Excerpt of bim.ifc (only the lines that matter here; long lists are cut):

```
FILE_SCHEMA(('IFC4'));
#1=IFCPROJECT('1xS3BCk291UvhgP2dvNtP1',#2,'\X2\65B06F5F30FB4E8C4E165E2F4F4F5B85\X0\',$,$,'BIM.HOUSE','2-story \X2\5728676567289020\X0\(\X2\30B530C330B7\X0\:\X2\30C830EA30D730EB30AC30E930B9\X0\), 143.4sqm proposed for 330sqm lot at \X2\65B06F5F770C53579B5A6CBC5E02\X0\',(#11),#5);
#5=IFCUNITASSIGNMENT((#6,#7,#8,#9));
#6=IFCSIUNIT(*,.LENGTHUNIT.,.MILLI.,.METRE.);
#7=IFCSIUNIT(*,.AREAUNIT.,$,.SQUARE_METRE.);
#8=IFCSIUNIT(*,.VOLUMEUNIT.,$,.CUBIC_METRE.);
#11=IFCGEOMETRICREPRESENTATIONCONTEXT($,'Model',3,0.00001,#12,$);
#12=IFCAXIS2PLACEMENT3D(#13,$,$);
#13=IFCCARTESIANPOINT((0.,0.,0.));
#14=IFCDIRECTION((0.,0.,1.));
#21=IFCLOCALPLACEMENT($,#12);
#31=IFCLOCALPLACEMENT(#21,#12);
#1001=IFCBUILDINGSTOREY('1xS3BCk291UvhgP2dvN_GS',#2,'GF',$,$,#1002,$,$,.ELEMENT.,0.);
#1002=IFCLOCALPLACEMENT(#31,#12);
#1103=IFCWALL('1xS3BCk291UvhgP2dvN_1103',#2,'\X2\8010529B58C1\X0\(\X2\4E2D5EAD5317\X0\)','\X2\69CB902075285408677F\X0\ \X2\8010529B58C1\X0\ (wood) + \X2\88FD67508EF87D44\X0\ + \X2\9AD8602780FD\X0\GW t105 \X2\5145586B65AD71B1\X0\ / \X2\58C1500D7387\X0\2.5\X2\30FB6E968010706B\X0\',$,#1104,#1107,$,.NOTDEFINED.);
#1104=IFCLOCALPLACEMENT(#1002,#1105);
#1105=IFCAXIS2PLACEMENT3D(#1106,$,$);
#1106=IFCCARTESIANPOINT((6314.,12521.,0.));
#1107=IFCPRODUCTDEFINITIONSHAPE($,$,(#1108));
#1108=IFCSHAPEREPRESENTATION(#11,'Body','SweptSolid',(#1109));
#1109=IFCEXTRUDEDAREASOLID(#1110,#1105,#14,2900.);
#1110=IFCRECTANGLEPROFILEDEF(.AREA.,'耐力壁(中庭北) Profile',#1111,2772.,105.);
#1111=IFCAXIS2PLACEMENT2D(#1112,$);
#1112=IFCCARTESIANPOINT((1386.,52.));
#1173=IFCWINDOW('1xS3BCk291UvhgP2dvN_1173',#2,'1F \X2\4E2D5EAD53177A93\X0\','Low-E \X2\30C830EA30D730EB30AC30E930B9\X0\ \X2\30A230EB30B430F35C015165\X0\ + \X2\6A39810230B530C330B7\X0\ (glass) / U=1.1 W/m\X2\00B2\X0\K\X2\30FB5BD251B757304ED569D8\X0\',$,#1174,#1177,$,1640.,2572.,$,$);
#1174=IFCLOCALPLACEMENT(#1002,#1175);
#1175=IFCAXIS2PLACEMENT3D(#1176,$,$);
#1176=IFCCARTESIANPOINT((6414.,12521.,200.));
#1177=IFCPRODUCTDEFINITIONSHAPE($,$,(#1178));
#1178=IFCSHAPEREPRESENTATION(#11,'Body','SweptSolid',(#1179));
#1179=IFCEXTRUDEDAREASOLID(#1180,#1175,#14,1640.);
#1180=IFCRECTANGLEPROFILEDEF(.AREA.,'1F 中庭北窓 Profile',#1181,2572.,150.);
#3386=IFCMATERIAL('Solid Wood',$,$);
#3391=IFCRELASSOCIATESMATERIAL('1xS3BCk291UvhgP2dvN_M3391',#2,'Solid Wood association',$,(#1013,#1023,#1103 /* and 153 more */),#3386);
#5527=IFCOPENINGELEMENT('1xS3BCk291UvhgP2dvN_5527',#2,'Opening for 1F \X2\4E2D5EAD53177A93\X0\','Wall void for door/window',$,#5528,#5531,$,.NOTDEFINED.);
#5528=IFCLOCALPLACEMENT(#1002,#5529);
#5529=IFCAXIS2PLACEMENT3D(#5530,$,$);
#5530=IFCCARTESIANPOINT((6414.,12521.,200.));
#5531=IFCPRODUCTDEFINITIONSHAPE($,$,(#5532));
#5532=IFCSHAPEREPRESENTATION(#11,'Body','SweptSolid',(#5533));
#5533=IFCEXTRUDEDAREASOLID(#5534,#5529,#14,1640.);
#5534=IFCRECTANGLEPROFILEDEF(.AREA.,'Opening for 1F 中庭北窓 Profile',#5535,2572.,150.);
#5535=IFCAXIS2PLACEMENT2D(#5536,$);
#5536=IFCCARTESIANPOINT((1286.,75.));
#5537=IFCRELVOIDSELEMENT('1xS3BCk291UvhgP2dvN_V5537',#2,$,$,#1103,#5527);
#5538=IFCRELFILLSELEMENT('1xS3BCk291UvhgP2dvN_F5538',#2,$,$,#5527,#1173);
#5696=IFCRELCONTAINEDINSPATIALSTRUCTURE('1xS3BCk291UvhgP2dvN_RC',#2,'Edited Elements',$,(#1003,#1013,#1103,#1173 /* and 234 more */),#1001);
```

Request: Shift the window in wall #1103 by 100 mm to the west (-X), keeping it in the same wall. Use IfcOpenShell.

```python
import ifcopenshell
import ifcopenshell.api.geometry
import ifcopenshell.util.placement
import ifcopenshell.util.unit

model = ifcopenshell.open("bim.ifc")
unit_scale = ifcopenshell.util.unit.calculate_unit_scale(model)

window = model.by_guid("1xS3BCk291UvhgP2dvN_1173")
opening = window.FillsVoids[0].RelatingOpeningElement
wall = opening.VoidsElements[0].RelatingBuildingElement

wall_matrix = ifcopenshell.util.placement.get_local_placement(wall.ObjectPlacement)
shift = wall_matrix[:3, 0] * -0.1 / unit_scale
before = ifcopenshell.util.placement.get_local_placement(window.ObjectPlacement)[:3, 3].copy()

# The window is not placed relative to its opening, so move both.
for product in (opening, window):
    matrix = ifcopenshell.util.placement.get_local_placement(product.ObjectPlacement)
    matrix[:3, 3] += shift
    ifcopenshell.api.geometry.edit_object_placement(model, product=product, matrix=matrix, is_si=False)

after = ifcopenshell.util.placement.get_local_placement(window.ObjectPlacement)[:3, 3]
print("window moved by", (after - before).round(3) + 0.0)

model.write("bim_v2.ifc")
```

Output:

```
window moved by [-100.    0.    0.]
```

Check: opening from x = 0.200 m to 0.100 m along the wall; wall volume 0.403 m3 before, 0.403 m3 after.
